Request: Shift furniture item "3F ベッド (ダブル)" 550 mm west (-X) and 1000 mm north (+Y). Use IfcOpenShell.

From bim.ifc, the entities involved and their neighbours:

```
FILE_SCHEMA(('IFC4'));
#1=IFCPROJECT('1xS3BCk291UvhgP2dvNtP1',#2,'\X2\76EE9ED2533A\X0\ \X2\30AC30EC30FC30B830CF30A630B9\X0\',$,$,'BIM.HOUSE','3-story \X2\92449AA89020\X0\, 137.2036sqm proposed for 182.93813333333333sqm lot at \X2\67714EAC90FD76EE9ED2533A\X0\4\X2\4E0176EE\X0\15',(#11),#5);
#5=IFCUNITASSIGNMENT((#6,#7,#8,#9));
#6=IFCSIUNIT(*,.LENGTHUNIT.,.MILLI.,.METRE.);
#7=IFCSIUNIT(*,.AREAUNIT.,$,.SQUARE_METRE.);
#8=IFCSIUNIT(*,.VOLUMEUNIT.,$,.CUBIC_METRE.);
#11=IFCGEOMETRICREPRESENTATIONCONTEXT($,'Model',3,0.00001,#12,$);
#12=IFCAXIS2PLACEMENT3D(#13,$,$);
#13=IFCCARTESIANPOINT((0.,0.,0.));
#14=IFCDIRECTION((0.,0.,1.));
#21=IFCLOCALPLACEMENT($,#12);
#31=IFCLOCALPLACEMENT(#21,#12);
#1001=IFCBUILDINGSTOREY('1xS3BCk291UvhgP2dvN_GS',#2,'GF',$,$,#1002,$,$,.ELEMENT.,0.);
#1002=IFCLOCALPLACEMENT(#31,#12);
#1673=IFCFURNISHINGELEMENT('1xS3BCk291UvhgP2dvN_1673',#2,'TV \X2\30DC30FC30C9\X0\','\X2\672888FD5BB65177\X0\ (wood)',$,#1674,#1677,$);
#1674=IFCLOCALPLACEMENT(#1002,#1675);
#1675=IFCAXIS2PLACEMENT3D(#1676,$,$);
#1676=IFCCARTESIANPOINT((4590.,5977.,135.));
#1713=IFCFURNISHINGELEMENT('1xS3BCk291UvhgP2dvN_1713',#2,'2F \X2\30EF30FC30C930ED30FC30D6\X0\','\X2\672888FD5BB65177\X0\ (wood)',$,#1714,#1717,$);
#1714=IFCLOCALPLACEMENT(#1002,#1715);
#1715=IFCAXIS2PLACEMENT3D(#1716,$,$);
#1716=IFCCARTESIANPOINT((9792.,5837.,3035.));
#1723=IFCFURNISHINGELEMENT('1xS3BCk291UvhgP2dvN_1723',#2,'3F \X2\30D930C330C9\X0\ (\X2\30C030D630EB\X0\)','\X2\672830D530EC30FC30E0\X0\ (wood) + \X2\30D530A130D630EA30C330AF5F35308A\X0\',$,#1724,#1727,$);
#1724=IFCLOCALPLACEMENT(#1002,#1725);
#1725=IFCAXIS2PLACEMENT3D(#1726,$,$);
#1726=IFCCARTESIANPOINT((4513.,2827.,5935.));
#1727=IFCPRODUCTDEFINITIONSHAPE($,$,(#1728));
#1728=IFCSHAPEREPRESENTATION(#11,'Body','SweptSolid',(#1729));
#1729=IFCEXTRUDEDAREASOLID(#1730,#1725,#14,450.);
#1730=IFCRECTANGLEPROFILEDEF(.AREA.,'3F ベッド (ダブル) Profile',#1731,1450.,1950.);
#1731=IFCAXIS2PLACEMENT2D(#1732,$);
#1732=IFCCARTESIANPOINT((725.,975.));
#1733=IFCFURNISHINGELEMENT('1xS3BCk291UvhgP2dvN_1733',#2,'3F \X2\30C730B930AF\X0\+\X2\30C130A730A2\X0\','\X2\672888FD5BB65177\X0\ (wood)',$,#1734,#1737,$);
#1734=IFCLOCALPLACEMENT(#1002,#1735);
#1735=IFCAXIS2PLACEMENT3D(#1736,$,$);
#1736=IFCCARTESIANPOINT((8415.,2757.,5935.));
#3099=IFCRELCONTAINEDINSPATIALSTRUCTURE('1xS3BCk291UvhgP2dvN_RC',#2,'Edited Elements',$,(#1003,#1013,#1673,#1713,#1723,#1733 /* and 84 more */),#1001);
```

```python
import ifcopenshell
import ifcopenshell.api.geometry
import ifcopenshell.util.placement

model = ifcopenshell.open("bim.ifc")

item = model.by_guid("1xS3BCk291UvhgP2dvN_1723")
matrix = ifcopenshell.util.placement.get_local_placement(item.ObjectPlacement)
matrix[0, 3] -= 550.0
matrix[1, 3] += 1000.0
ifcopenshell.api.geometry.edit_object_placement(model, product=item, matrix=matrix, is_si=False)

print(ifcopenshell.util.placement.get_local_placement(item.ObjectPlacement).round(3) + 0.0)

model.write("bim_updated.ifc")
```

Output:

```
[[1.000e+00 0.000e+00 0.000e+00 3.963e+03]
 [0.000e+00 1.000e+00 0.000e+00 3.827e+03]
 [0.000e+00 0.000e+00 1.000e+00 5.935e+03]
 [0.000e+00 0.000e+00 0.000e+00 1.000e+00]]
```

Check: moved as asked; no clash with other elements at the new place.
